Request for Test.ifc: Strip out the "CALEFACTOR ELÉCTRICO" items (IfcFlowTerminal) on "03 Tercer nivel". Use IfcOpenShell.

First a look at what the model holds.

```python
import ifcopenshell
import ifcopenshell.util.element

model = ifcopenshell.open("Test.ifc")
print(model.schema)
storey = next(s for s in model.by_type("IfcBuildingStorey") if s.Name == "03 Tercer nivel")
terminals = [e for e in ifcopenshell.util.element.get_decomposition(storey) if e.is_a("IfcFlowTerminal")]
seen = {}
for e in terminals:
    element_type = ifcopenshell.util.element.get_type(e)
    name = element_type.Name if element_type not in (None, e) else None
    seen[name] = seen.get(name, 0) + 1
for name, count in sorted(seen.items(), key=str):
    print(count, "x", name)
```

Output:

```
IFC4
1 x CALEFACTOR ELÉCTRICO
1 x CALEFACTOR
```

```python
import ifcopenshell
import ifcopenshell.api.root
import ifcopenshell.util.element

model = ifcopenshell.open("Test.ifc")

storey = next(s for s in model.by_type("IfcBuildingStorey") if s.Name == "03 Tercer nivel")
terminals = [e for e in ifcopenshell.util.element.get_decomposition(storey) if e.is_a("IfcFlowTerminal")]
targets = [e for e in terminals if (t := ifcopenshell.util.element.get_type(e)) not in (None, e) and t.Name == "CALEFACTOR ELÉCTRICO"]

for e in targets:
    ifcopenshell.api.root.remove_product(model, product=e)
print(len(targets), "removed")

model.write("Test-out.ifc")
```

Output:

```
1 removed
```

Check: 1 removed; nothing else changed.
